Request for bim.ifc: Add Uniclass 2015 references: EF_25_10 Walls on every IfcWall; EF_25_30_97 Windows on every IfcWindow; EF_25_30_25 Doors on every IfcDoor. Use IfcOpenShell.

First a look at what the model holds.

```python
import ifcopenshell

model = ifcopenshell.open("bim.ifc")
print(model.schema)
print("classifications:", [c.Name for c in model.by_type("IfcClassification")])
for ifc_class in ("IfcDoor", "IfcRoof", "IfcStair", "IfcWall", "IfcWindow"):
    print(ifc_class, len(model.by_type(ifc_class)))
```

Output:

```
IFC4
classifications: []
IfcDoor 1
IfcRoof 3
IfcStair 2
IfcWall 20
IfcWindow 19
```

```python
import ifcopenshell
import ifcopenshell.api.classification

model = ifcopenshell.open("bim.ifc")

system = ifcopenshell.api.classification.add_classification(model, classification="Uniclass 2015")

codes = {
    "IfcWall": ("EF_25_10", "Walls"),
    "IfcWindow": ("EF_25_30_97", "Windows"),
    "IfcDoor": ("EF_25_30_25", "Doors"),
}
for ifc_class, (code, name) in codes.items():
    products = model.by_type(ifc_class)
    ifcopenshell.api.classification.add_reference(
        model, products=products, classification=system, identification=code, name=name
    )
    print(code, len(products))

model.write("bim_v2.ifc")
```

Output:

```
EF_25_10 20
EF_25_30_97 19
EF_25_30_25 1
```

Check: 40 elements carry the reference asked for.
